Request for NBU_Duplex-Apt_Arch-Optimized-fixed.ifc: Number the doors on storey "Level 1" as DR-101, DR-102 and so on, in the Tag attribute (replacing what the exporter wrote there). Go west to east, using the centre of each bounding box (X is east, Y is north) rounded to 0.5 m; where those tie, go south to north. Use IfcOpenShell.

First a look at what the model holds.

```python
import ifcopenshell
import ifcopenshell.util.element
import ifcopenshell.util.placement

model = ifcopenshell.open("NBU_Duplex-Apt_Arch-Optimized-fixed.ifc")
print(model.schema)
storey = next(s for s in model.by_type("IfcBuildingStorey") if s.Name == "Level 1")
doors = [e for e in ifcopenshell.util.element.get_decomposition(storey) if e.is_a("IfcDoor")]
for e in sorted(doors, key=lambda e: e.id()):
    origin = ifcopenshell.util.placement.get_local_placement(e.ObjectPlacement)[:3, 3]
    print(e.id(), e.Tag, e.Name, origin.round(2) + 0.0, sep=" | ")
```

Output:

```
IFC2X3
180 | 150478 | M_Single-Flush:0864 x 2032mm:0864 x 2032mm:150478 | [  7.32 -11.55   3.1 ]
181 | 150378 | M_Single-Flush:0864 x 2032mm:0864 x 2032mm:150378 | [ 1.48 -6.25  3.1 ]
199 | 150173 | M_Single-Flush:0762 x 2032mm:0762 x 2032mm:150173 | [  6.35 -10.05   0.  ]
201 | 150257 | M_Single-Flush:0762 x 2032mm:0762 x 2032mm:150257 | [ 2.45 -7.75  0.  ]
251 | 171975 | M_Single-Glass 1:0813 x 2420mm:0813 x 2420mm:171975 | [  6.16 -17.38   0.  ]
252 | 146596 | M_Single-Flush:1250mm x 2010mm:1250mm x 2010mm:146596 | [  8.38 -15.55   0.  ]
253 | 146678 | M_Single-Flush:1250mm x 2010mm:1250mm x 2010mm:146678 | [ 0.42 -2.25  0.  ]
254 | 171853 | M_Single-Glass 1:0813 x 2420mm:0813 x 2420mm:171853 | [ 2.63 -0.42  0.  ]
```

```python
import ifcopenshell
import ifcopenshell.geom
import ifcopenshell.util.element
import ifcopenshell.util.shape

model = ifcopenshell.open("NBU_Duplex-Apt_Arch-Optimized-fixed.ifc")
settings = ifcopenshell.geom.settings()
settings.set("use-world-coords", True)


def centre(element):
    shape = ifcopenshell.geom.create_shape(settings, element)
    return ifcopenshell.util.shape.get_bbox_centroid(shape.geometry)


storey = next(s for s in model.by_type("IfcBuildingStorey") if s.Name == "Level 1")
doors = [e for e in ifcopenshell.util.element.get_decomposition(storey) if e.is_a("IfcDoor")]

# Insertion points can sit at a corner or the storey origin, so sort by the geometry (in metres).
centres = {e: centre(e) for e in doors}
doors.sort(key=lambda e: (round(centres[e][0] / 0.5), centres[e][1]))

for i, e in enumerate(doors, start=1):
    number = f"DR-1{i:02d}"
    e.Tag = number
    print(e.id(), number)

model.write("NBU_Duplex-Apt_Arch-Optimized-fixed-out.ifc")
```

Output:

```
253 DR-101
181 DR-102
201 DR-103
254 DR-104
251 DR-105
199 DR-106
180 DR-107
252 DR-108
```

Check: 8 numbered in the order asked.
